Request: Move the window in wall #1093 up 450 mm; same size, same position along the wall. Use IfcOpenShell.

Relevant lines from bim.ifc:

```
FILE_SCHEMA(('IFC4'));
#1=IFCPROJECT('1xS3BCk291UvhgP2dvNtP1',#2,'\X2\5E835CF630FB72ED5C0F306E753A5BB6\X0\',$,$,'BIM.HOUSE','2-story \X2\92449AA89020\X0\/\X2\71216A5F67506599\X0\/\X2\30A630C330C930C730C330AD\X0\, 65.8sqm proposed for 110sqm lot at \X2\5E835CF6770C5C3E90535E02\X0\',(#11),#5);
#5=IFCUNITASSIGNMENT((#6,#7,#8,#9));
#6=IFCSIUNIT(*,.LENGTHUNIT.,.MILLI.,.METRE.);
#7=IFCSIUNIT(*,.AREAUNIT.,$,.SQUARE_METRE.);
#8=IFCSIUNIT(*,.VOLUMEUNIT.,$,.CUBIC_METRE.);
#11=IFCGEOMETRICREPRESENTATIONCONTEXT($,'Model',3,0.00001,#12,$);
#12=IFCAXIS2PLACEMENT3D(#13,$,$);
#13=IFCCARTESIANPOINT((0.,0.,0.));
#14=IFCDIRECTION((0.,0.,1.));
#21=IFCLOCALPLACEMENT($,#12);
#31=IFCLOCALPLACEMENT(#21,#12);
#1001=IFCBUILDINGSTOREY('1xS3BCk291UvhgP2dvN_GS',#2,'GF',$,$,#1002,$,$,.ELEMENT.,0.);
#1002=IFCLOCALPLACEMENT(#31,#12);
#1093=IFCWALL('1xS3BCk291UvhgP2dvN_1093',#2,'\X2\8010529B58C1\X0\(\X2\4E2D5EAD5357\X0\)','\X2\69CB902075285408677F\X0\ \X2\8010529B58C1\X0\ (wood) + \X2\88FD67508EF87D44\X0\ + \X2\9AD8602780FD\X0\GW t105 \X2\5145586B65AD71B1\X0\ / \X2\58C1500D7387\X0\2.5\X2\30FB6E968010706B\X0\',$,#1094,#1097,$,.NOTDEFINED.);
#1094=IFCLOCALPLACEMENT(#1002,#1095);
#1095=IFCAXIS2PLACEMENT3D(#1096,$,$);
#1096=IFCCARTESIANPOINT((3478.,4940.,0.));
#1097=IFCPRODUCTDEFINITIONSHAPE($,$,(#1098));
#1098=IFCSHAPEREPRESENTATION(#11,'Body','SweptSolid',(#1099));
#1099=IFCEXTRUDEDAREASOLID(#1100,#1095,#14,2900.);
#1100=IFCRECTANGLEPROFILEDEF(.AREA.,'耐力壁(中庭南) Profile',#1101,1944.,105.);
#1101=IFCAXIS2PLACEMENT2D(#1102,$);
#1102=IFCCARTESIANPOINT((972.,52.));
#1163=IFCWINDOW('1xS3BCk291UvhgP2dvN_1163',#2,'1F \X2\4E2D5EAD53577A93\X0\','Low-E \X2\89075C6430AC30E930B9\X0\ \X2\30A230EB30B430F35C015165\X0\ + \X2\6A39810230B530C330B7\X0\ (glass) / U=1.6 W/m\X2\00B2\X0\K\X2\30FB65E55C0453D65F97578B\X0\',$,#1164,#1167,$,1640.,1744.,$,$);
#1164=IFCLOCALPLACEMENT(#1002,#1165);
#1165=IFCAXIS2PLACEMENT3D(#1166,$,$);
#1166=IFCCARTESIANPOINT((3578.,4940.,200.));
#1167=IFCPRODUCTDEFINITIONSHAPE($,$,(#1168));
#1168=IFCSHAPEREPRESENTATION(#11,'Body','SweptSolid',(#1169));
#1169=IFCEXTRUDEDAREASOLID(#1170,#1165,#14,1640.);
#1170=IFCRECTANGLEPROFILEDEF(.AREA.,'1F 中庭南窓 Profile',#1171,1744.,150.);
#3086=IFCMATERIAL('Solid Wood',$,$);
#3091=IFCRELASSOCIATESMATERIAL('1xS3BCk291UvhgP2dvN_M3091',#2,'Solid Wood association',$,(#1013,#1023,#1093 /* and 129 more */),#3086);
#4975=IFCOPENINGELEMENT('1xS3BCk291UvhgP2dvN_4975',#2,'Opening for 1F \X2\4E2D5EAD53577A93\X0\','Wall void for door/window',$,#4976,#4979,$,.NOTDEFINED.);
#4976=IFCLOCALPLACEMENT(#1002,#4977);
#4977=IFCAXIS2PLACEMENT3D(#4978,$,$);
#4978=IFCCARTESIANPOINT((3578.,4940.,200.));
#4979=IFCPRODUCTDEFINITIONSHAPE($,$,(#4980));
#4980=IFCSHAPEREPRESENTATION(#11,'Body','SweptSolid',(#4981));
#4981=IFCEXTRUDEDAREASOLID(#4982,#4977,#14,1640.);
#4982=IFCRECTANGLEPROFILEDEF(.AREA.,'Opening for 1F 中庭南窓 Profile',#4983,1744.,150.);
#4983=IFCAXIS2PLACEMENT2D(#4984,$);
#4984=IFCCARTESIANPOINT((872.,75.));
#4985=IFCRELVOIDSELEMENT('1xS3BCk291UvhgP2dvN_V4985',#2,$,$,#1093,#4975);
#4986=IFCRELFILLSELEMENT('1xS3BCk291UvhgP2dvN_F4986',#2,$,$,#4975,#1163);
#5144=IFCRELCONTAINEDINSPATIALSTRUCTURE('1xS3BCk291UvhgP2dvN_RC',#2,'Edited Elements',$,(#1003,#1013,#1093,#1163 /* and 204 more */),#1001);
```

```python
import numpy as np
import ifcopenshell
import ifcopenshell.api.geometry
import ifcopenshell.util.placement
import ifcopenshell.util.unit

model = ifcopenshell.open("bim.ifc")
unit_scale = ifcopenshell.util.unit.calculate_unit_scale(model)

window = model.by_id(1163)
opening = window.FillsVoids[0].RelatingOpeningElement
dz = 0.45 / unit_scale

shift = np.array([0.0, 0.0, dz])
# The window is not placed relative to its opening, so move both.
for product in (opening, window):
    matrix = ifcopenshell.util.placement.get_local_placement(product.ObjectPlacement)
    matrix[:3, 3] += shift
    ifcopenshell.api.geometry.edit_object_placement(model, product=product, matrix=matrix, is_si=False)

print(f"moved by {dz * unit_scale:+.3f} m")

model.write("bim_v2.ifc")
```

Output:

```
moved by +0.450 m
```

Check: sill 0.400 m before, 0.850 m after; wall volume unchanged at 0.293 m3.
